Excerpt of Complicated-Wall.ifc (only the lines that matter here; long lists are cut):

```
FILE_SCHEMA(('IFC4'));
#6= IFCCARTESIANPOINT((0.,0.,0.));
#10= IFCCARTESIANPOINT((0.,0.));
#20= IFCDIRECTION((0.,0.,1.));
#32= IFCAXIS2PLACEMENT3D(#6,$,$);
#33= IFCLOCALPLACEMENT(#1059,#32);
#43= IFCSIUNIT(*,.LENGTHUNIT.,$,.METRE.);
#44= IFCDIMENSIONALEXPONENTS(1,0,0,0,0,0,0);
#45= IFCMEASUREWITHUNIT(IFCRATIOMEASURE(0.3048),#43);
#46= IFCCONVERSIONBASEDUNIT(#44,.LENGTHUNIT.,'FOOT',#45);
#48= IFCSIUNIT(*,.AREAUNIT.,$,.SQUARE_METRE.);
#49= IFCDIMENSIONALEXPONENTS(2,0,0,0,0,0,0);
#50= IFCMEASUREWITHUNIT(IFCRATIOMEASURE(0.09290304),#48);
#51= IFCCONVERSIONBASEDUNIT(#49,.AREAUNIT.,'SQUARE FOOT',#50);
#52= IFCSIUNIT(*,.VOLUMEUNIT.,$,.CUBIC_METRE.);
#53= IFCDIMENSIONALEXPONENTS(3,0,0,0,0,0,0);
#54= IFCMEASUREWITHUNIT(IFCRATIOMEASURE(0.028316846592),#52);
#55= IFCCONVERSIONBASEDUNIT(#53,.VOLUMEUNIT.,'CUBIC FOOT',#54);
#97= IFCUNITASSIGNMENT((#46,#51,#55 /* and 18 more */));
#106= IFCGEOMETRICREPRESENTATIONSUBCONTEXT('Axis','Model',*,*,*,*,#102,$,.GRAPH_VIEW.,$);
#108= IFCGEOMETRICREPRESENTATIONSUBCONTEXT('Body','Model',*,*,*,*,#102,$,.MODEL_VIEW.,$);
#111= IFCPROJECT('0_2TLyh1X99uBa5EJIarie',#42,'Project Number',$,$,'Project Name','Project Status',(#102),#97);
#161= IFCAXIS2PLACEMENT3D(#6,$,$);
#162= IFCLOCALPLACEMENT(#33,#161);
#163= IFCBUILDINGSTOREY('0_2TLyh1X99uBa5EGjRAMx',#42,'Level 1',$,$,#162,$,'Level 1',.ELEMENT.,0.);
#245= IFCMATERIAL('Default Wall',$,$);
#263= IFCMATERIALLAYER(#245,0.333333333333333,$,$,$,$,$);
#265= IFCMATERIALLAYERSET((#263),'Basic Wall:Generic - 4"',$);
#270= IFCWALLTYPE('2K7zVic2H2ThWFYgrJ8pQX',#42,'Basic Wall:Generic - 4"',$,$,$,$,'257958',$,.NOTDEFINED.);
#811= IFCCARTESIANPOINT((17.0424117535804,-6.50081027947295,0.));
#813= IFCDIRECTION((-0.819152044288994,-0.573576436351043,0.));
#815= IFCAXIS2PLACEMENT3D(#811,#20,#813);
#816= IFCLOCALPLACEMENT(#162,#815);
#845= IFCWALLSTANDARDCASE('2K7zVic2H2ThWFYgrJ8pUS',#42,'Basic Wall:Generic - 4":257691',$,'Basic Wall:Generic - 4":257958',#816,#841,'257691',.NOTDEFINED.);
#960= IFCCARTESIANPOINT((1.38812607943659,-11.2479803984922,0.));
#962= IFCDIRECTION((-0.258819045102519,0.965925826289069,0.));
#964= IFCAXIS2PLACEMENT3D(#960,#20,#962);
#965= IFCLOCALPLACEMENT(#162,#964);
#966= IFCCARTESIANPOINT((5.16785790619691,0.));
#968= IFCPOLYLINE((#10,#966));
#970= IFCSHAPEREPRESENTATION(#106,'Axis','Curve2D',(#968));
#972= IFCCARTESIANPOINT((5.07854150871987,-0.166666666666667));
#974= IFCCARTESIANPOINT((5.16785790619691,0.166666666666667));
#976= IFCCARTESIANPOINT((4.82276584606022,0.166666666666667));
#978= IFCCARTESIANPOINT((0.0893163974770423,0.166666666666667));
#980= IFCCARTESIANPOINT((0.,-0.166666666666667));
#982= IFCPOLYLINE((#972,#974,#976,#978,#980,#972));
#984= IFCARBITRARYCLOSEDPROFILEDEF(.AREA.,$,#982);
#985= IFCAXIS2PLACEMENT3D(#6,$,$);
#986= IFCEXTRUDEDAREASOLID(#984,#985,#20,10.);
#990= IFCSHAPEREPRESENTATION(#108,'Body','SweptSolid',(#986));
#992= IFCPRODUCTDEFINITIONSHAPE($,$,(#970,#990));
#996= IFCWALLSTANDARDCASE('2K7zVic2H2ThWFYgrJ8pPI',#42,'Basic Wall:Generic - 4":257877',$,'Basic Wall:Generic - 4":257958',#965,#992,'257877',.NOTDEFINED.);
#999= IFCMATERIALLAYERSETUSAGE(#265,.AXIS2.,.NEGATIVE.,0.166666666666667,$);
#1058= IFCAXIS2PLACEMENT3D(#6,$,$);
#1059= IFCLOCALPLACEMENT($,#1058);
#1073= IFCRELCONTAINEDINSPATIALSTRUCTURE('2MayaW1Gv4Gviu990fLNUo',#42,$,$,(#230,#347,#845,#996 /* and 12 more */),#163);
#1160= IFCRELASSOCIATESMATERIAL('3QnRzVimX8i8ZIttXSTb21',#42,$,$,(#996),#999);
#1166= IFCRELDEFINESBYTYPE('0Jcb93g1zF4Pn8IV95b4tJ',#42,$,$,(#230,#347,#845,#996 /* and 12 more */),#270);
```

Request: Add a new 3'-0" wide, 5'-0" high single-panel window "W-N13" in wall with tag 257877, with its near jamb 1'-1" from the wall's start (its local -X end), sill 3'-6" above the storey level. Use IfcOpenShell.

```python
import numpy as np
import ifcopenshell
import ifcopenshell.api.feature
import ifcopenshell.api.geometry
import ifcopenshell.api.root
import ifcopenshell.api.spatial
import ifcopenshell.geom
import ifcopenshell.util.element
import ifcopenshell.util.placement
import ifcopenshell.util.representation
import ifcopenshell.util.shape
import ifcopenshell.util.unit

model = ifcopenshell.open("Complicated-Wall.ifc")
unit_scale = ifcopenshell.util.unit.calculate_unit_scale(model)
settings = ifcopenshell.geom.settings()


def volume(element):
    """Net volume in cubic metres, openings subtracted."""
    shape = ifcopenshell.geom.create_shape(settings, element)
    return ifcopenshell.util.shape.get_volume(shape.geometry)


wall = model.by_guid("2K7zVic2H2ThWFYgrJ8pPI")
storey = ifcopenshell.util.element.get_container(wall, ifc_class="IfcBuildingStorey")
context = ifcopenshell.util.representation.get_context(model, "Model", "Body", "MODEL_VIEW")
before = volume(wall)

width, height, from_end, sill = 0.9144, 1.524, 0.3302, 1.0668  # metres

# The wall runs along its own X axis, and the end named is its -X end.
wall_shape = ifcopenshell.geom.create_shape(settings, wall)
x, y, z = ifcopenshell.util.shape.get_vertices(wall_shape.geometry).T
start = x.min() + from_end
face, thickness = float(y.min()), float(y.max() - y.min())
wall_matrix = ifcopenshell.util.placement.get_local_placement(wall.ObjectPlacement)
level = ifcopenshell.util.placement.get_local_placement(storey.ObjectPlacement)[2, 3]


def in_wall(x, y):
    """Placement at x, y metres in the wall's axes, at sill height."""
    matrix = wall_matrix.copy()
    matrix[:, 3] = wall_matrix @ np.array([x / unit_scale, y / unit_scale, 0.0, 1.0])
    matrix[2, 3] = level + sill / unit_scale
    return matrix


# Opening: a box that overshoots both wall faces by 50 mm.
opening = ifcopenshell.api.root.create_entity(model, ifc_class="IfcOpeningElement", predefined_type="OPENING")
box = ifcopenshell.api.geometry.add_wall_representation(
    model, context=context, length=width, height=height, thickness=thickness + 0.1
)
ifcopenshell.api.geometry.assign_representation(model, product=opening, representation=box)
ifcopenshell.api.geometry.edit_object_placement(model, product=opening, matrix=in_wall(start, face - 0.05), is_si=False)
ifcopenshell.api.feature.add_feature(model, feature=opening, element=wall)

window = ifcopenshell.api.root.create_entity(model, ifc_class="IfcWindow", name="W-N13", predefined_type="WINDOW")
window.OverallWidth, window.OverallHeight = width / unit_scale, height / unit_scale
window.PartitioningType = "SINGLE_PANEL"
body = ifcopenshell.api.geometry.add_window_representation(
    model,
    context=context,
    overall_width=window.OverallWidth,
    overall_height=window.OverallHeight,
    partition_type="SINGLE_PANEL",
)
ifcopenshell.api.geometry.assign_representation(model, product=window, representation=body)
ifcopenshell.api.spatial.assign_container(model, products=[window], relating_structure=storey)
ifcopenshell.api.feature.add_filling(model, opening=opening, element=window)

# Centre the window in the wall's thickness.
ifcopenshell.api.geometry.edit_object_placement(model, product=window, matrix=in_wall(start, face), is_si=False)
window_shape = ifcopenshell.geom.create_shape(settings, window)
depth = ifcopenshell.util.shape.get_vertices(window_shape.geometry)[:, 1]
offset = face + thickness / 2 - (depth.min() + depth.max()) / 2
ifcopenshell.api.geometry.edit_object_placement(model, product=window, matrix=in_wall(start, offset), is_si=False)

after = volume(wall)

print(f"wall volume {before:.3f} -> {after:.3f} m3")

model.write("Complicated-Wall_updated.ifc")
```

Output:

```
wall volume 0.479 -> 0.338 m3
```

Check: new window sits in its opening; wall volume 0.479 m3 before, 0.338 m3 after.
